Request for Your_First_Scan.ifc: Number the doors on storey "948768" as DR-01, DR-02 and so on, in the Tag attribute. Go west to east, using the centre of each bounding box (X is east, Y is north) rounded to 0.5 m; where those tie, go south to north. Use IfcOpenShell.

First a look at what the model holds.

```python
import ifcopenshell
import ifcopenshell.util.element
import ifcopenshell.util.placement

model = ifcopenshell.open("Your_First_Scan.ifc")
print(model.schema)
storey = next(s for s in model.by_type("IfcBuildingStorey") if s.Name == "948768")
doors = [e for e in ifcopenshell.util.element.get_decomposition(storey) if e.is_a("IfcDoor")]
for e in sorted(doors, key=lambda e: e.id()):
    origin = ifcopenshell.util.placement.get_local_placement(e.ObjectPlacement)[:3, 3]
    print(e.id(), e.Tag, e.Name, origin.round(2) + 0.0, sep=" | ")
```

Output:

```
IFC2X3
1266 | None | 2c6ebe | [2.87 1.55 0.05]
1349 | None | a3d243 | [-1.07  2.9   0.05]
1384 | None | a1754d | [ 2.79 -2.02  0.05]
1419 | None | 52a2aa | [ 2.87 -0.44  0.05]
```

```python
import ifcopenshell
import ifcopenshell.geom
import ifcopenshell.util.element
import ifcopenshell.util.shape

model = ifcopenshell.open("Your_First_Scan.ifc")
settings = ifcopenshell.geom.settings()
settings.set("use-world-coords", True)


def centre(element):
    shape = ifcopenshell.geom.create_shape(settings, element)
    return ifcopenshell.util.shape.get_bbox_centroid(shape.geometry)


storey = next(s for s in model.by_type("IfcBuildingStorey") if s.Name == "948768")
doors = [e for e in ifcopenshell.util.element.get_decomposition(storey) if e.is_a("IfcDoor")]

# Insertion points can sit at a corner or the storey origin, so sort by the geometry (in metres).
centres = {e: centre(e) for e in doors}
doors.sort(key=lambda e: (round(centres[e][0] / 0.5), centres[e][1]))

for i, e in enumerate(doors, start=1):
    number = f"DR-{i:02d}"
    e.Tag = number
    print(e.id(), number)

model.write("Your_First_Scan_updated.ifc")
```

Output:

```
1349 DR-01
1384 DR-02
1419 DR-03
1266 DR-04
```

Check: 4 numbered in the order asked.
